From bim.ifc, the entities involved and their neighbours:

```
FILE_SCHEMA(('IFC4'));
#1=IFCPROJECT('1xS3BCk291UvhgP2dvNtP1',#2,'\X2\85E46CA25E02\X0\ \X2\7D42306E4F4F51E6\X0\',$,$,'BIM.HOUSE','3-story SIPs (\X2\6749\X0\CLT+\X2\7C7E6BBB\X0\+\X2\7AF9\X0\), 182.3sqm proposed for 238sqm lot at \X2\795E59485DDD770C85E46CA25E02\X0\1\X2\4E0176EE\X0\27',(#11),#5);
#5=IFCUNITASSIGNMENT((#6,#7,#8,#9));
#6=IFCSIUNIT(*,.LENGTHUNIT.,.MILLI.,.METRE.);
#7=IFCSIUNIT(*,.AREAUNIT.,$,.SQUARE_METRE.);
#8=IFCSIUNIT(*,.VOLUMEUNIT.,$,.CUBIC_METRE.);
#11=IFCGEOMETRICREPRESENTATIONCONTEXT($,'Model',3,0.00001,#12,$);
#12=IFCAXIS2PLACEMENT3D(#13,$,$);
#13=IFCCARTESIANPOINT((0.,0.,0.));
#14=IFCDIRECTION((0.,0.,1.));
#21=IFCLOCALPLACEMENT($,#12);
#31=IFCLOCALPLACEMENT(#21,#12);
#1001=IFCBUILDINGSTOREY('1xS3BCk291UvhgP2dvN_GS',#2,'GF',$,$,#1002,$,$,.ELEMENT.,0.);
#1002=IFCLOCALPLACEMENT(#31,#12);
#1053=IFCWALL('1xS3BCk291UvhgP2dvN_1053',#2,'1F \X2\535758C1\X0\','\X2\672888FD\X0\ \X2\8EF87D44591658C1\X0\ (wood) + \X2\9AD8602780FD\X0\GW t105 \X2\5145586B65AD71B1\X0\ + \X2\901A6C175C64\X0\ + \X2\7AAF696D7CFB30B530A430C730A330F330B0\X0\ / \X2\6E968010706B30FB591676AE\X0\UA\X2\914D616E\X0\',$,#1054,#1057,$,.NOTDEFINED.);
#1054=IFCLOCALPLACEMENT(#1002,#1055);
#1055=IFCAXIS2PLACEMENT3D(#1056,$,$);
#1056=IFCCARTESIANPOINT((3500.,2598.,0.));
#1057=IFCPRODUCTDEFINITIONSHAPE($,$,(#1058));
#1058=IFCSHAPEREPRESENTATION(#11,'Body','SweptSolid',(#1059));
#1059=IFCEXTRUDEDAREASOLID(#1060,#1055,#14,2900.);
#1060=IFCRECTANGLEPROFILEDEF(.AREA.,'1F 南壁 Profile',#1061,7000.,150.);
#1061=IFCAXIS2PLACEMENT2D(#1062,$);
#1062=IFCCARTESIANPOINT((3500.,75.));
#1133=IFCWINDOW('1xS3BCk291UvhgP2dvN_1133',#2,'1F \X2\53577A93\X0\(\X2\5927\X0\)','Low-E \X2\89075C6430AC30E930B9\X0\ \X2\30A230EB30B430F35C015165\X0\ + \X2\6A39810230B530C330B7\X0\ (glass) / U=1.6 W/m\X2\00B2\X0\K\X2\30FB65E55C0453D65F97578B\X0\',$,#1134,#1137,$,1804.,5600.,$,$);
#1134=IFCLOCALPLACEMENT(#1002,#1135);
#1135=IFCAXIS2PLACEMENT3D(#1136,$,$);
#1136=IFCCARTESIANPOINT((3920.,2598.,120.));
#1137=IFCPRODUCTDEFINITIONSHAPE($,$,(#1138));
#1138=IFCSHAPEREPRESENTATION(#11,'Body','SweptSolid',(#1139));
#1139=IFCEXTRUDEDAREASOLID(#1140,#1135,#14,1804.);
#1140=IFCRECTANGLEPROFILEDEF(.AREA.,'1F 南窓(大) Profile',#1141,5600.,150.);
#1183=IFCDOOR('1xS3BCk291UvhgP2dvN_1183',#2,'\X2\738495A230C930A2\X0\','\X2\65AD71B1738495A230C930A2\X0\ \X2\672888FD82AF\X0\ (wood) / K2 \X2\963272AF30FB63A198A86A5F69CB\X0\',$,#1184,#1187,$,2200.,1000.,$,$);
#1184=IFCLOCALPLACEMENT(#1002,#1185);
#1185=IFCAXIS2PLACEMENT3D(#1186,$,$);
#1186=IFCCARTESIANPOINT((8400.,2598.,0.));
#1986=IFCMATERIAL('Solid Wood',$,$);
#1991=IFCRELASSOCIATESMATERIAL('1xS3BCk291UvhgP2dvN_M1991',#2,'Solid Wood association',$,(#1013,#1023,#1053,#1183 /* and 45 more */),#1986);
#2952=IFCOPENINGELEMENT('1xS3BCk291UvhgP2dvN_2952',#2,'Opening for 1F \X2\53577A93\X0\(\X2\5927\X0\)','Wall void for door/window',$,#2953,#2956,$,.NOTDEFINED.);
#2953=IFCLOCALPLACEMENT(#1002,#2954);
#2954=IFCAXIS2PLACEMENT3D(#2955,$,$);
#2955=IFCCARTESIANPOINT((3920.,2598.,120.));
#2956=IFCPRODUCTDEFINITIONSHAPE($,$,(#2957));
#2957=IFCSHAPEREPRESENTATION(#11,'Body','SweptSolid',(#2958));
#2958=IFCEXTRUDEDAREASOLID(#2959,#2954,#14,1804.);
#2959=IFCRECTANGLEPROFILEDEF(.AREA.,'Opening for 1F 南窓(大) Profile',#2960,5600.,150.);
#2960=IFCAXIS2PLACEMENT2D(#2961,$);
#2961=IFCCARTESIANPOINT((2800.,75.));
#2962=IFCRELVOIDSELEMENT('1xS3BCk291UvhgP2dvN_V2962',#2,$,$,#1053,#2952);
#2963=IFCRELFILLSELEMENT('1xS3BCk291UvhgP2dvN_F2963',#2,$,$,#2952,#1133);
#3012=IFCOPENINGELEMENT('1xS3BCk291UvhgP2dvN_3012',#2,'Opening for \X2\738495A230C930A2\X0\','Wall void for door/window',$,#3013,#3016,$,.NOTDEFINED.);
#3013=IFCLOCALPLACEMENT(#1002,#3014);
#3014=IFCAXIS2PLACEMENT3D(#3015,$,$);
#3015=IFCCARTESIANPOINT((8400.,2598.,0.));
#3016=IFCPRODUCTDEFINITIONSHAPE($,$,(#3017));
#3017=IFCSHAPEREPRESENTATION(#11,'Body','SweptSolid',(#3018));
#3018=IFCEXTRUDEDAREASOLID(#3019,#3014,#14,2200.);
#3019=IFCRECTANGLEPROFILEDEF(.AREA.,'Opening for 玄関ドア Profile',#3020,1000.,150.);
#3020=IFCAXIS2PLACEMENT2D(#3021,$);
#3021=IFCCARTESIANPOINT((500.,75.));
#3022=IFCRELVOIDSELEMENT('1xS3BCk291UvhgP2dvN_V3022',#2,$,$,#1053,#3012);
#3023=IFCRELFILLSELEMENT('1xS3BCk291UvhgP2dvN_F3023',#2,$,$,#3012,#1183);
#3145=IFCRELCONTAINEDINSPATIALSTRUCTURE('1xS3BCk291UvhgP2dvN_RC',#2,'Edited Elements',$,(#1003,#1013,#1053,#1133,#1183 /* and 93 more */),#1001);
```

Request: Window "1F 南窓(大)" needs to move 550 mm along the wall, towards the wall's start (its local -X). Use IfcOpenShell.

```python
import ifcopenshell
import ifcopenshell.api.geometry
import ifcopenshell.util.placement
import ifcopenshell.util.unit

model = ifcopenshell.open("bim.ifc")
unit_scale = ifcopenshell.util.unit.calculate_unit_scale(model)

window = model.by_id(1133)
opening = window.FillsVoids[0].RelatingOpeningElement
wall = opening.VoidsElements[0].RelatingBuildingElement

wall_matrix = ifcopenshell.util.placement.get_local_placement(wall.ObjectPlacement)
shift = wall_matrix[:3, 0] * -0.55 / unit_scale
before = ifcopenshell.util.placement.get_local_placement(window.ObjectPlacement)[:3, 3].copy()

# The window is not placed relative to its opening, so move both.
for product in (opening, window):
    matrix = ifcopenshell.util.placement.get_local_placement(product.ObjectPlacement)
    matrix[:3, 3] += shift
    ifcopenshell.api.geometry.edit_object_placement(model, product=product, matrix=matrix, is_si=False)

after = ifcopenshell.util.placement.get_local_placement(window.ObjectPlacement)[:3, 3]
print("window moved by", (after - before).round(3) + 0.0)

model.write("bim-out.ifc")
```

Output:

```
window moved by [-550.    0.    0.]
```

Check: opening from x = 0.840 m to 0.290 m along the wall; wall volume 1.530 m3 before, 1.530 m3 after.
